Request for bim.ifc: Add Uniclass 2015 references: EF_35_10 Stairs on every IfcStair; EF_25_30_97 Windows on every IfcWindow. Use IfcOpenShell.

First a look at what the model holds.

```python
import ifcopenshell

model = ifcopenshell.open("bim.ifc")
print(model.schema)
print("classifications:", [c.Name for c in model.by_type("IfcClassification")])
for ifc_class in ("IfcDoor", "IfcRoof", "IfcStair", "IfcWall", "IfcWindow"):
    print(ifc_class, len(model.by_type(ifc_class)))
```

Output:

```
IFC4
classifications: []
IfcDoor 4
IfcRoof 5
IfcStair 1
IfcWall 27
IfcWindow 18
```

```python
import ifcopenshell
import ifcopenshell.api.classification

model = ifcopenshell.open("bim.ifc")

system = ifcopenshell.api.classification.add_classification(model, classification="Uniclass 2015")

codes = {
    "IfcStair": ("EF_35_10", "Stairs"),
    "IfcWindow": ("EF_25_30_97", "Windows"),
}
for ifc_class, (code, name) in codes.items():
    products = model.by_type(ifc_class)
    ifcopenshell.api.classification.add_reference(
        model, products=products, classification=system, identification=code, name=name
    )
    print(code, len(products))

model.write("bim-out.ifc")
```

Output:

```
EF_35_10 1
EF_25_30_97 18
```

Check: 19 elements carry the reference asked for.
